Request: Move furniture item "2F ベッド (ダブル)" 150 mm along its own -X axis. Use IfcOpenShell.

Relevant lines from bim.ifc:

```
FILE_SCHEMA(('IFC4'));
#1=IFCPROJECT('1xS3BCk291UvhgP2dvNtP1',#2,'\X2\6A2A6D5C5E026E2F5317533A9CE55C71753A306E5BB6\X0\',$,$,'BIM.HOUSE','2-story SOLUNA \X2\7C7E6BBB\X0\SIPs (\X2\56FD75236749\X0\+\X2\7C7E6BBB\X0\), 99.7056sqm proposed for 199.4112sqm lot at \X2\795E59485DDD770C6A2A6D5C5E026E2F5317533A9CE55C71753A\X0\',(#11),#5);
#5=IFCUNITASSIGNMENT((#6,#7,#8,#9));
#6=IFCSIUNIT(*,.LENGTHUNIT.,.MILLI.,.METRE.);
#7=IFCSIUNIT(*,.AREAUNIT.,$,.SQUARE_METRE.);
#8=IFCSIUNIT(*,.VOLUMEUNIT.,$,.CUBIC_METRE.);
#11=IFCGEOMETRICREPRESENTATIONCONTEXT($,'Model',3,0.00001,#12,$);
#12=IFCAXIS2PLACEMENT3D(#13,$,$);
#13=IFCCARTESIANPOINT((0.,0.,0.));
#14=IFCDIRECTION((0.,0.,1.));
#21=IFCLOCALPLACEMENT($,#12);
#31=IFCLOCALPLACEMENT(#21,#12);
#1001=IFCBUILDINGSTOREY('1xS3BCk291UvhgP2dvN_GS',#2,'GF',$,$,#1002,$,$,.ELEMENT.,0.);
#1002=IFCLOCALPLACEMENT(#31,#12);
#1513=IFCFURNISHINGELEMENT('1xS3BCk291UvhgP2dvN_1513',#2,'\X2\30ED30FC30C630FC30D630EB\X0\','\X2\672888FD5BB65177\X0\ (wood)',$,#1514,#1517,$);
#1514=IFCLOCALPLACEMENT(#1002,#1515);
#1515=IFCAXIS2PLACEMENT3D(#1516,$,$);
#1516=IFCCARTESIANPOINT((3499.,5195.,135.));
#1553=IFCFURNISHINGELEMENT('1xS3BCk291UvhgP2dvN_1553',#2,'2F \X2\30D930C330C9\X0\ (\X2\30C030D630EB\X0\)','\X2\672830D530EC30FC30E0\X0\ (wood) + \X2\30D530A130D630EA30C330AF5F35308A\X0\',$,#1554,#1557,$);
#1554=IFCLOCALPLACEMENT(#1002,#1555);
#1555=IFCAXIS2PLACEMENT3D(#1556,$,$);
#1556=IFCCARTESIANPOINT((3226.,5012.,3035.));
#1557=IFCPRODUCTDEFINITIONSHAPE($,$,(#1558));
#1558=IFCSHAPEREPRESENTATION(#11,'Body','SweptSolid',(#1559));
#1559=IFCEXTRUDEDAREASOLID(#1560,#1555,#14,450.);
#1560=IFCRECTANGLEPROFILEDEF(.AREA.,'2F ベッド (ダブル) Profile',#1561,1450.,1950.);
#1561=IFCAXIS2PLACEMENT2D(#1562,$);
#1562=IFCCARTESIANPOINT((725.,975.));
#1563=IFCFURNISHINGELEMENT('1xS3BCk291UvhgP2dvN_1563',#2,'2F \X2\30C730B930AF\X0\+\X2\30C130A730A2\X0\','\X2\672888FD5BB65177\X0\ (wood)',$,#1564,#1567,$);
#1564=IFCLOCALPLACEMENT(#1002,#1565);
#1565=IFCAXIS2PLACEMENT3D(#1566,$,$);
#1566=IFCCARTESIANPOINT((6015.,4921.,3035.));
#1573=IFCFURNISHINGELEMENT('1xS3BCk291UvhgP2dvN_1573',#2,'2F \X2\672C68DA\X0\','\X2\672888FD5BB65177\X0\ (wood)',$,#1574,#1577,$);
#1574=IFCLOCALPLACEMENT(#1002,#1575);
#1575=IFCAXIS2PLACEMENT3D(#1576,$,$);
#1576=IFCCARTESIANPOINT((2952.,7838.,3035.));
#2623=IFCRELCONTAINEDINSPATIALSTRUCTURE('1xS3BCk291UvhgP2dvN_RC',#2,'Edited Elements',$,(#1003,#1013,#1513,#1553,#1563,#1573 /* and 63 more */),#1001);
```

```python
import ifcopenshell
import ifcopenshell.api.geometry
import ifcopenshell.util.placement
import ifcopenshell.util.unit

model = ifcopenshell.open("bim.ifc")
unit_scale = ifcopenshell.util.unit.calculate_unit_scale(model)

item = model.by_guid("1xS3BCk291UvhgP2dvN_1553")
matrix = ifcopenshell.util.placement.get_local_placement(item.ObjectPlacement)
matrix[:3, 3] -= matrix[:3, 0] * 0.15 / unit_scale
ifcopenshell.api.geometry.edit_object_placement(model, product=item, matrix=matrix, is_si=False)

print(ifcopenshell.util.placement.get_local_placement(item.ObjectPlacement).round(3) + 0.0)

model.write("bim-out.ifc")
```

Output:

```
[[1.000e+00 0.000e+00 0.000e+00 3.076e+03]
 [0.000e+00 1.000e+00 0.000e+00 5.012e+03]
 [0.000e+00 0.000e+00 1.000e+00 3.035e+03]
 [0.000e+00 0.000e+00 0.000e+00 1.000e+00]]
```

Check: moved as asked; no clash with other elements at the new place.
